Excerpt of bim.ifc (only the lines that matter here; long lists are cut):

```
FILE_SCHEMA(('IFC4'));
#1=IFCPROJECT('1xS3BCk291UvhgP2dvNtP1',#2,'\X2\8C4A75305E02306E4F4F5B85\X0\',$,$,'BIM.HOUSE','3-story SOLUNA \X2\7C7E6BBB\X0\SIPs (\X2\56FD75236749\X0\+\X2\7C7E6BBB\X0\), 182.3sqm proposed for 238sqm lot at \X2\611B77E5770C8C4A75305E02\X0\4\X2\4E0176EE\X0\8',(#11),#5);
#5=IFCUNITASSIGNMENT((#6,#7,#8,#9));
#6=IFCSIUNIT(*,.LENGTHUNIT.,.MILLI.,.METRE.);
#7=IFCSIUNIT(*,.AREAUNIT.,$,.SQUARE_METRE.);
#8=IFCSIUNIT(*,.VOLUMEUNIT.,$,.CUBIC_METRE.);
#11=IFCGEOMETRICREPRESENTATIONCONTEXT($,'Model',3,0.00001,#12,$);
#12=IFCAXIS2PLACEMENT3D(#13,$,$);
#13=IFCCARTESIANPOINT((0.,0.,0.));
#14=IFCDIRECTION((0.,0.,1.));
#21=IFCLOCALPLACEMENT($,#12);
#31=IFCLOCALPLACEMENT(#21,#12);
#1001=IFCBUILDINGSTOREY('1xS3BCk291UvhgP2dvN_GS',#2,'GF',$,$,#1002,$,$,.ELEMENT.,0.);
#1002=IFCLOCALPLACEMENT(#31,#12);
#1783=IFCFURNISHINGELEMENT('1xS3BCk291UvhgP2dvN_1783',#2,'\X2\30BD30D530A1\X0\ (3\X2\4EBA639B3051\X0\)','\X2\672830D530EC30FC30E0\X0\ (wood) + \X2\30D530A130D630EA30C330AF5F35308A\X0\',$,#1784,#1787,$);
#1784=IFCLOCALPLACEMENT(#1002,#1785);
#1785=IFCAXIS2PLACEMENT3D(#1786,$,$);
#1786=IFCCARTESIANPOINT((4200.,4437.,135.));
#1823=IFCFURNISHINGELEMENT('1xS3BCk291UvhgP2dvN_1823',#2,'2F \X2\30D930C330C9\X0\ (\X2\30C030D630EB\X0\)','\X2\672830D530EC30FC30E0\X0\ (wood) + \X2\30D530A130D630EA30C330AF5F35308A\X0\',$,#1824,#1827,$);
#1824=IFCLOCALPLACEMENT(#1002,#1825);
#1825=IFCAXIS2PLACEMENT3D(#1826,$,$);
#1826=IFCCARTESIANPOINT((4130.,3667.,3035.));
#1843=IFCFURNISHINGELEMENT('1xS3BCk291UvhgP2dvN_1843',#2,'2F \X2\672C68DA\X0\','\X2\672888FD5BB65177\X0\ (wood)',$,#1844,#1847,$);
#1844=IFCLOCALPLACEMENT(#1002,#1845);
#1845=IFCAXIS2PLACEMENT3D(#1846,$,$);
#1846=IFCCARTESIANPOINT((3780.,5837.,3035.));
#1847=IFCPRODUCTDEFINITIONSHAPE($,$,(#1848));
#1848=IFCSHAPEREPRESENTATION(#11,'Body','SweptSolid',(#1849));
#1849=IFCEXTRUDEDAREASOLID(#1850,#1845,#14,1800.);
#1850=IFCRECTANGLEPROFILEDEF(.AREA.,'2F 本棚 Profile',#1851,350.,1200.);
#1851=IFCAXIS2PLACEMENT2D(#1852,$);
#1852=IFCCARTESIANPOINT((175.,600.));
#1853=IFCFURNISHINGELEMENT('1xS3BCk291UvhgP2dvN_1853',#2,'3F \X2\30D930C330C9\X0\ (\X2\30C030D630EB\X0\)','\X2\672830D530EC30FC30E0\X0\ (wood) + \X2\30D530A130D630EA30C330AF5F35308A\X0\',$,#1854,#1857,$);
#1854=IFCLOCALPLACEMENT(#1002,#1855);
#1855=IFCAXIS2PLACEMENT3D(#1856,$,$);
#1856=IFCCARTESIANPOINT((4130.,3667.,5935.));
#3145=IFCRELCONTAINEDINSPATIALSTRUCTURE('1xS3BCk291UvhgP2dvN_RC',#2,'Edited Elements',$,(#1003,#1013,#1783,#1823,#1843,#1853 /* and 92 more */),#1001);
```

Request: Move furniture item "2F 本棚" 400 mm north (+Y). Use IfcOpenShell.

```python
import ifcopenshell
import ifcopenshell.api.geometry
import ifcopenshell.util.placement

model = ifcopenshell.open("bim.ifc")

item = model.by_guid("1xS3BCk291UvhgP2dvN_1843")
matrix = ifcopenshell.util.placement.get_local_placement(item.ObjectPlacement)
matrix[1, 3] += 400.0
ifcopenshell.api.geometry.edit_object_placement(model, product=item, matrix=matrix, is_si=False)

print(ifcopenshell.util.placement.get_local_placement(item.ObjectPlacement).round(3) + 0.0)

model.write("bim_v2.ifc")
```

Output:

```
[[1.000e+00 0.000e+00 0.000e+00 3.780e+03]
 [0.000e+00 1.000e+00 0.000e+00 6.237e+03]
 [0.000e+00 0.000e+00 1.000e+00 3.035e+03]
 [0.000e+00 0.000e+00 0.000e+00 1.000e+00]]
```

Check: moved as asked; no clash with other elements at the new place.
